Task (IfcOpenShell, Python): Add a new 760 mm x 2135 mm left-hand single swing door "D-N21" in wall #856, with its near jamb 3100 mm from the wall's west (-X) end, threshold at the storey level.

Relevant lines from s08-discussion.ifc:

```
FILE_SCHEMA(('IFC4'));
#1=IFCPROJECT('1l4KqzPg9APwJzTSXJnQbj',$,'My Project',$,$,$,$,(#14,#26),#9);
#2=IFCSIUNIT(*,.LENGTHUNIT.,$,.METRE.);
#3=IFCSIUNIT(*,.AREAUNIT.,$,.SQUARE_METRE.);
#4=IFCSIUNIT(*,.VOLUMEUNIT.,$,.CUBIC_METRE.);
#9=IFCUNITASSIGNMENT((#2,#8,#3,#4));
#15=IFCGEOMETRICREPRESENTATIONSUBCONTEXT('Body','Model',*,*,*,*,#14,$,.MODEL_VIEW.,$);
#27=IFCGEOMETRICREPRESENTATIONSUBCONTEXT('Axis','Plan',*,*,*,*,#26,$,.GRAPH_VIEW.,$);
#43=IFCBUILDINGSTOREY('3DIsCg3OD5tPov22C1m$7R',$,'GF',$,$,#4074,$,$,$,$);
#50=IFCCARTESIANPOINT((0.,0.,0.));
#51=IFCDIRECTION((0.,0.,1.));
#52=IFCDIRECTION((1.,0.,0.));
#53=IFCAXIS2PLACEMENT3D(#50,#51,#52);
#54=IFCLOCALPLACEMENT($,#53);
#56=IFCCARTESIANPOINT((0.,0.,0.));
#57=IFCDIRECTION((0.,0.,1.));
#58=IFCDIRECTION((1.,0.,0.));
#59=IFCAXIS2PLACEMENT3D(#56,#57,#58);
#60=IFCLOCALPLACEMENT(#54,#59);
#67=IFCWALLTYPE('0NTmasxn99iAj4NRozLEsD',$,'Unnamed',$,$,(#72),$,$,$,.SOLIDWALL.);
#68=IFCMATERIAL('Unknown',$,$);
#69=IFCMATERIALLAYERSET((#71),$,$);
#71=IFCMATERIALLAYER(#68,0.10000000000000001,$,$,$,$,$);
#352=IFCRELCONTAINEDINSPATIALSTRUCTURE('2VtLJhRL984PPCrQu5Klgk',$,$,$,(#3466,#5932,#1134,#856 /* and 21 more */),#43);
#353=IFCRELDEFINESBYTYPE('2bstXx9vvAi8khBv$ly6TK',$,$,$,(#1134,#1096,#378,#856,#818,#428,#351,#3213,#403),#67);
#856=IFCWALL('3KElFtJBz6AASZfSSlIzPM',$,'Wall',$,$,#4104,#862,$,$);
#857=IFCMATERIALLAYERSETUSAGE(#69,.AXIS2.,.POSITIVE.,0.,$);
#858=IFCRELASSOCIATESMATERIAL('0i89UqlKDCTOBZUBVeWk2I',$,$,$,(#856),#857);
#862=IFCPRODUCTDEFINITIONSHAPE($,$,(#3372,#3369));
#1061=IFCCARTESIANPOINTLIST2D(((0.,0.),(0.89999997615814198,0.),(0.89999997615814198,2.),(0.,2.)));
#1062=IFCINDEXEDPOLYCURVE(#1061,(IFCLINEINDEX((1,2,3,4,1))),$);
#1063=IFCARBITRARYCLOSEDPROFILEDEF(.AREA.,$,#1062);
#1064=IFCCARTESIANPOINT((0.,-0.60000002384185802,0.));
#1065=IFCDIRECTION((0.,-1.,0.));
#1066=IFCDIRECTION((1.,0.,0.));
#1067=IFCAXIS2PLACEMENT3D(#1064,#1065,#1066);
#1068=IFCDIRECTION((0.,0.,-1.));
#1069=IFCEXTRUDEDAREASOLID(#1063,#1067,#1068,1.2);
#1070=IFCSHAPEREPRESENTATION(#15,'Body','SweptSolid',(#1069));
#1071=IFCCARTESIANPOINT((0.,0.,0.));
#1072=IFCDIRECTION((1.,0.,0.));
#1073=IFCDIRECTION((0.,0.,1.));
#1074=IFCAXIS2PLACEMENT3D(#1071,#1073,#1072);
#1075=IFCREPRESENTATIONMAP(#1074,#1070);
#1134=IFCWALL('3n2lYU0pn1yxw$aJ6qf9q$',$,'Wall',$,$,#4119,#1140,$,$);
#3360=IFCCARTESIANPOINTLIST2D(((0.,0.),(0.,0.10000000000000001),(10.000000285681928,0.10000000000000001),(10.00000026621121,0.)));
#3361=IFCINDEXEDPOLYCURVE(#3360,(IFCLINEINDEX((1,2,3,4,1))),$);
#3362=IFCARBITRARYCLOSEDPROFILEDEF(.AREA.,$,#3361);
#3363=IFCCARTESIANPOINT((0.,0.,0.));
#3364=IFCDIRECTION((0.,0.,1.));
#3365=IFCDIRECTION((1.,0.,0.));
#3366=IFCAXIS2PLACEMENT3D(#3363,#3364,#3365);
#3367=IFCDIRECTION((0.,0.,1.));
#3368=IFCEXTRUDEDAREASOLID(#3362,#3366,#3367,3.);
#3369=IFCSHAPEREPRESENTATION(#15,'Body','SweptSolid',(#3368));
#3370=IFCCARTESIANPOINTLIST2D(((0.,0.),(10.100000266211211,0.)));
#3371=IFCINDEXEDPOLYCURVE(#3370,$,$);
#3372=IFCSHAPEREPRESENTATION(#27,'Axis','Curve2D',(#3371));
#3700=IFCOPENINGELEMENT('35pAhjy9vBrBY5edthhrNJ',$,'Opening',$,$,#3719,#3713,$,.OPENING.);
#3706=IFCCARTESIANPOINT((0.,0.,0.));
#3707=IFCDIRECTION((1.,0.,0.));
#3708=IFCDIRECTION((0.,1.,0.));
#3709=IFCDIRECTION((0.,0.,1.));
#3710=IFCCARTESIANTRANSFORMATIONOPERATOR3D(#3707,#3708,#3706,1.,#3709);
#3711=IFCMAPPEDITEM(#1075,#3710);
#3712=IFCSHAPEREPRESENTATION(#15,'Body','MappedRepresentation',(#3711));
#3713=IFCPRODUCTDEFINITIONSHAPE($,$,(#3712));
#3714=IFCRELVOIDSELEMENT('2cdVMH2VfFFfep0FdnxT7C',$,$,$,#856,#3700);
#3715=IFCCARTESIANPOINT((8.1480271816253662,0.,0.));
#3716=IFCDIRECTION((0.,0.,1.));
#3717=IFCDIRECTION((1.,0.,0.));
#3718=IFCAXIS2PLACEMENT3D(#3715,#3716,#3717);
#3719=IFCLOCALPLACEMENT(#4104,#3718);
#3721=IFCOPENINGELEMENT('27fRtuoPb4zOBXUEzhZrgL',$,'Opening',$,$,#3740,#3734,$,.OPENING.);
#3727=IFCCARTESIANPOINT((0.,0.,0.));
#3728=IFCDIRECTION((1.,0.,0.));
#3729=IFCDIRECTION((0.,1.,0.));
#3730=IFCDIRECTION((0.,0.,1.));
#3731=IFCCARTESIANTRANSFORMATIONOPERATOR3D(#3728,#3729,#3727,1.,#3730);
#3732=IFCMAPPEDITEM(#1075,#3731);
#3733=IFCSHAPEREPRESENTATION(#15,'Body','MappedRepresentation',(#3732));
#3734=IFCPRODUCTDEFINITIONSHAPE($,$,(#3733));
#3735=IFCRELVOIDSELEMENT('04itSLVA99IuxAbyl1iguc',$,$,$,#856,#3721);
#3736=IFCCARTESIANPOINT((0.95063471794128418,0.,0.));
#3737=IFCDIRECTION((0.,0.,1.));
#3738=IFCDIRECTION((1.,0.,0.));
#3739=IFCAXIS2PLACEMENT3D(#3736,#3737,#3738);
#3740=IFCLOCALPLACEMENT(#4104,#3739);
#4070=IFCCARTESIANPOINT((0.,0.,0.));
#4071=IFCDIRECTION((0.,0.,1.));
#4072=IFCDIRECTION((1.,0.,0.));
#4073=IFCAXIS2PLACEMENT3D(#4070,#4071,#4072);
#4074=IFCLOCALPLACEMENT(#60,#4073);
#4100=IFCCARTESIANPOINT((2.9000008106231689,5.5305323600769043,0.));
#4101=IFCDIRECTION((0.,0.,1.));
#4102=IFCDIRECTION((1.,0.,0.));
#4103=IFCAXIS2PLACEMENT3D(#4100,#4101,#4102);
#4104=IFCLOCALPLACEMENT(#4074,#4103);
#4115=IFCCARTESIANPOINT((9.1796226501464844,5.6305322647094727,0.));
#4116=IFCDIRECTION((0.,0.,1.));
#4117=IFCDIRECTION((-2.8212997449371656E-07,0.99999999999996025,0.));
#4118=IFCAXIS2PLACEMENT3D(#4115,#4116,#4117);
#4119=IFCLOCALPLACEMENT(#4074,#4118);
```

```python
import numpy as np
import ifcopenshell
import ifcopenshell.api.feature
import ifcopenshell.api.geometry
import ifcopenshell.api.root
import ifcopenshell.api.spatial
import ifcopenshell.geom
import ifcopenshell.util.element
import ifcopenshell.util.placement
import ifcopenshell.util.representation
import ifcopenshell.util.shape
import ifcopenshell.util.unit

model = ifcopenshell.open("s08-discussion.ifc")
unit_scale = ifcopenshell.util.unit.calculate_unit_scale(model)
settings = ifcopenshell.geom.settings()


def volume(element):
    """Net volume in cubic metres, openings subtracted."""
    shape = ifcopenshell.geom.create_shape(settings, element)
    return ifcopenshell.util.shape.get_volume(shape.geometry)


wall = model.by_guid("3KElFtJBz6AASZfSSlIzPM")
storey = ifcopenshell.util.element.get_container(wall, ifc_class="IfcBuildingStorey")
context = ifcopenshell.util.representation.get_context(model, "Model", "Body", "MODEL_VIEW")
before = volume(wall)

width, height, from_end, sill = 0.76, 2.135, 3.1, 0.0  # metres

# The wall runs along its own X axis, and the end named is its -X end.
wall_shape = ifcopenshell.geom.create_shape(settings, wall)
x, y, z = ifcopenshell.util.shape.get_vertices(wall_shape.geometry).T
start = x.min() + from_end
face, thickness = float(y.min()), float(y.max() - y.min())
wall_matrix = ifcopenshell.util.placement.get_local_placement(wall.ObjectPlacement)
level = ifcopenshell.util.placement.get_local_placement(storey.ObjectPlacement)[2, 3]


def in_wall(x, y):
    """Placement at x, y metres in the wall's axes, at sill height."""
    matrix = wall_matrix.copy()
    matrix[:, 3] = wall_matrix @ np.array([x / unit_scale, y / unit_scale, 0.0, 1.0])
    matrix[2, 3] = level + sill / unit_scale
    return matrix


# Opening: a box that overshoots both wall faces by 50 mm.
opening = ifcopenshell.api.root.create_entity(model, ifc_class="IfcOpeningElement", predefined_type="OPENING")
box = ifcopenshell.api.geometry.add_wall_representation(
    model, context=context, length=width, height=height, thickness=thickness + 0.1
)
ifcopenshell.api.geometry.assign_representation(model, product=opening, representation=box)
ifcopenshell.api.geometry.edit_object_placement(model, product=opening, matrix=in_wall(start, face - 0.05), is_si=False)
ifcopenshell.api.feature.add_feature(model, feature=opening, element=wall)

door = ifcopenshell.api.root.create_entity(model, ifc_class="IfcDoor", name="D-N21", predefined_type="DOOR")
door.OverallWidth, door.OverallHeight = width / unit_scale, height / unit_scale
door.OperationType = "SINGLE_SWING_LEFT"
body = ifcopenshell.api.geometry.add_door_representation(
    model,
    context=context,
    overall_width=door.OverallWidth,
    overall_height=door.OverallHeight,
    operation_type="SINGLE_SWING_LEFT",
    lining_properties={"LiningDepth": thickness / unit_scale, "ThresholdDepth": thickness / unit_scale},
)
ifcopenshell.api.geometry.assign_representation(model, product=door, representation=body)
ifcopenshell.api.spatial.assign_container(model, products=[door], relating_structure=storey)
ifcopenshell.api.feature.add_filling(model, opening=opening, element=door)

# The lining spans the wall, so the door starts at the wall face.
ifcopenshell.api.geometry.edit_object_placement(model, product=door, matrix=in_wall(start, face), is_si=False)

after = volume(wall)

print(f"wall volume {before:.3f} -> {after:.3f} m3")

model.write("s08-discussion_edited.ifc")
```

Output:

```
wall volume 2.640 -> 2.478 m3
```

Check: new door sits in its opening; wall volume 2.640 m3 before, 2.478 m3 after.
